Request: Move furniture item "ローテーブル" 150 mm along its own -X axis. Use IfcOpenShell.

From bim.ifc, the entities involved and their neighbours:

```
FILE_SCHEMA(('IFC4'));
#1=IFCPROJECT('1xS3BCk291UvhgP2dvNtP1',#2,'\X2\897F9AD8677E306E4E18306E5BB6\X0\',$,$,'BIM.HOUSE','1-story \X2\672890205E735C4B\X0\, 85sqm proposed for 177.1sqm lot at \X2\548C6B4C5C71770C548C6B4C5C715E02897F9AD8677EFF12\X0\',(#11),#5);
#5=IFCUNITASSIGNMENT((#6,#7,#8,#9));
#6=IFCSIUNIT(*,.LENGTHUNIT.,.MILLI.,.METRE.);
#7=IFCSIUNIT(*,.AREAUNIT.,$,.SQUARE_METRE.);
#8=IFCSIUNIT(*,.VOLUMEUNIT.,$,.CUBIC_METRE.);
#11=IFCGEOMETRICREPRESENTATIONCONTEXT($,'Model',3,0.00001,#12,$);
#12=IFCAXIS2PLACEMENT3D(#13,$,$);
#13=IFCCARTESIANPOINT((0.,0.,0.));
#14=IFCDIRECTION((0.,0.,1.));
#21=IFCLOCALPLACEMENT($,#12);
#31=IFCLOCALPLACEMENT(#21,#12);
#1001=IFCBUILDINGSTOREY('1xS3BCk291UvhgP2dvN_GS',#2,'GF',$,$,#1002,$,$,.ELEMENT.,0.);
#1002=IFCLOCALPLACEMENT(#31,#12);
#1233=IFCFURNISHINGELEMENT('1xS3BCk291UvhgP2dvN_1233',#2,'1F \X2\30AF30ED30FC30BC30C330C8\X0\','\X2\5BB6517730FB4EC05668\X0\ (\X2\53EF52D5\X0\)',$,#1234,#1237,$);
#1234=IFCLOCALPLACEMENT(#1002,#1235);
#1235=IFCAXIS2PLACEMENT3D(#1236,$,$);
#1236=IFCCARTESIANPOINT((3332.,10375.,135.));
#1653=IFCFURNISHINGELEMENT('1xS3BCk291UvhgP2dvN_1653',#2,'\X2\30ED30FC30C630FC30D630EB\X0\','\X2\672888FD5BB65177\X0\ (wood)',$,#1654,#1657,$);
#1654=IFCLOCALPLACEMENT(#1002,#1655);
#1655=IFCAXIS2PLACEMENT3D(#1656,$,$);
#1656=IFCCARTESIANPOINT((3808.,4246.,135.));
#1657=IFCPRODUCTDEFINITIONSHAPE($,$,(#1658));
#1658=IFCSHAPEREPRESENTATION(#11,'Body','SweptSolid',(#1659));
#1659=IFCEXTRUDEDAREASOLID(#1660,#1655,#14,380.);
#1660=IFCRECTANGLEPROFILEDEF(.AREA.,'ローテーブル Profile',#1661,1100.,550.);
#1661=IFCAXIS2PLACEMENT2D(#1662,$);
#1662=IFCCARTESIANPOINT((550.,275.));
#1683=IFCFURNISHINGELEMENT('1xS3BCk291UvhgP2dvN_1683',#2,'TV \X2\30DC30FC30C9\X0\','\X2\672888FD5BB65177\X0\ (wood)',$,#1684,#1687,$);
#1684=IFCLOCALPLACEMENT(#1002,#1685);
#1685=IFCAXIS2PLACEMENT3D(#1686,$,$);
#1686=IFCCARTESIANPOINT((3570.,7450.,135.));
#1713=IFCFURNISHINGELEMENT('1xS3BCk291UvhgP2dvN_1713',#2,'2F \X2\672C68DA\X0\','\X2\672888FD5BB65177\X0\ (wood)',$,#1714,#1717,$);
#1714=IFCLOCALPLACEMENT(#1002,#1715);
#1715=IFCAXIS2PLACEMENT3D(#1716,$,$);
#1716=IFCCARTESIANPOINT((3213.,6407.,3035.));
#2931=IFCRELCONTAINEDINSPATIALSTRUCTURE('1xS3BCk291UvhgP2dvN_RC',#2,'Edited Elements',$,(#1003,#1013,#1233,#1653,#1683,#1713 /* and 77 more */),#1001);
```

```python
import ifcopenshell
import ifcopenshell.api.geometry
import ifcopenshell.util.placement

model = ifcopenshell.open("bim.ifc")

item = model.by_guid("1xS3BCk291UvhgP2dvN_1653")
matrix = ifcopenshell.util.placement.get_local_placement(item.ObjectPlacement)
matrix[:3, 3] -= matrix[:3, 0] * 150.0
ifcopenshell.api.geometry.edit_object_placement(model, product=item, matrix=matrix, is_si=False)

print(ifcopenshell.util.placement.get_local_placement(item.ObjectPlacement).round(3) + 0.0)

model.write("bim-out.ifc")
```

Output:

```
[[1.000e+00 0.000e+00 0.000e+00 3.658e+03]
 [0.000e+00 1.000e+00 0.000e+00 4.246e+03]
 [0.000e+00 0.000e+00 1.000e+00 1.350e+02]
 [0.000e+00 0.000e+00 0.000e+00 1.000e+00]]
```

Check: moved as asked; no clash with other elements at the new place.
